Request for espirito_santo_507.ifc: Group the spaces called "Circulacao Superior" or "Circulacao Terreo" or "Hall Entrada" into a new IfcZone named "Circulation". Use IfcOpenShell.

First a look at what the model holds.

```python
import ifcopenshell

model = ifcopenshell.open("espirito_santo_507.ifc")
print(model.schema)
seen = {}
for space in model.by_type("IfcSpace"):
    seen[space.Name] = seen.get(space.Name, 0) + 1
for name, count in sorted(seen.items(), key=str):
    print(count, "x", name)
print("zones:", [z.Name for z in model.by_type("IfcZone")][:20])
```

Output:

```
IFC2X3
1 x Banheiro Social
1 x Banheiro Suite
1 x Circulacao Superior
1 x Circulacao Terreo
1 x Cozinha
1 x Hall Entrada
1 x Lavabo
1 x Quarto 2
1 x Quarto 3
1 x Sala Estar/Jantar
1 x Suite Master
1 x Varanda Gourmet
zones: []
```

```python
import ifcopenshell
import ifcopenshell.api.group
import ifcopenshell.api.root

model = ifcopenshell.open("espirito_santo_507.ifc")

names = {"Circulacao Superior", "Circulacao Terreo", "Hall Entrada"}
spaces = [s for s in model.by_type("IfcSpace") if s.Name in names]

zone = ifcopenshell.api.root.create_entity(model, ifc_class="IfcZone", name="Circulation")
ifcopenshell.api.group.assign_group(model, products=spaces, group=zone)
print(len(spaces), "spaces in", zone.Name)

model.write("espirito_santo_507_edited.ifc")
```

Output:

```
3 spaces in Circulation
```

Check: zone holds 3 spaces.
